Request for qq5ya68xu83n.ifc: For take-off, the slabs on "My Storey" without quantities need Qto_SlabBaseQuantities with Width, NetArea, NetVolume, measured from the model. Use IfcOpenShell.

First a look at what the model holds.

```python
import ifcopenshell
import ifcopenshell.util.element
import ifcopenshell.util.unit

model = ifcopenshell.open("qq5ya68xu83n.ifc")
print(model.schema)
for unit_type in ("LENGTHUNIT", "AREAUNIT", "VOLUMEUNIT"):
    print(unit_type, ifcopenshell.util.unit.calculate_unit_scale(model, unit_type))
storey = next(s for s in model.by_type("IfcBuildingStorey") if s.Name == "My Storey")
slabs = [e for e in ifcopenshell.util.element.get_decomposition(storey) if e.is_a("IfcSlab")]
for e in sorted(slabs, key=lambda e: e.id()):
    print(e.id(), e.is_a(), e.Name, list(ifcopenshell.util.element.get_psets(e, qtos_only=True)), sep=" | ")
```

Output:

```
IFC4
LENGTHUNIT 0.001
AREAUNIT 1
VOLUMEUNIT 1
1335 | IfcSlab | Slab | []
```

```python
import ifcopenshell
import ifcopenshell.api.pset
import ifcopenshell.geom
import ifcopenshell.util.element
import ifcopenshell.util.shape
import ifcopenshell.util.unit

model = ifcopenshell.open("qq5ya68xu83n.ifc")
unit_scale = ifcopenshell.util.unit.calculate_unit_scale(model)
area_scale = ifcopenshell.util.unit.calculate_unit_scale(model, "AREAUNIT")
volume_scale = ifcopenshell.util.unit.calculate_unit_scale(model, "VOLUMEUNIT")
settings = ifcopenshell.geom.settings()

storey = next(s for s in model.by_type("IfcBuildingStorey") if s.Name == "My Storey")
slabs = [e for e in ifcopenshell.util.element.get_decomposition(storey) if e.is_a("IfcSlab")]

for e in sorted(slabs, key=lambda e: e.id()):
    if ifcopenshell.util.element.get_psets(e, qtos_only=True, should_inherit=False):
        continue
    # Geometry comes back in metres, in the element's own axes.
    shape = ifcopenshell.geom.create_shape(settings, e)
    values = {
        "Width": ifcopenshell.util.shape.get_z(shape.geometry) / unit_scale,
        "NetArea": ifcopenshell.util.shape.get_footprint_area(shape.geometry) / area_scale,
        "NetVolume": ifcopenshell.util.shape.get_volume(shape.geometry) / volume_scale,
    }
    qto = ifcopenshell.api.pset.add_qto(model, product=e, name="Qto_SlabBaseQuantities")
    ifcopenshell.api.pset.edit_qto(model, qto=qto, properties=values)
    print(e.id(), {k: round(v, 3) for k, v in values.items()})

model.write("qq5ya68xu83n-out.ifc")
```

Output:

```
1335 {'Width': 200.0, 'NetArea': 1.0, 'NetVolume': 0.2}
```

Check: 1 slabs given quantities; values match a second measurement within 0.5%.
